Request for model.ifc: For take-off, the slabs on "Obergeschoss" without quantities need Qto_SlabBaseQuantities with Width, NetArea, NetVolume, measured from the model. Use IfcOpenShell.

First a look at what the model holds.

```python
import ifcopenshell
import ifcopenshell.util.element
import ifcopenshell.util.unit

model = ifcopenshell.open("model.ifc")
print(model.schema)
for unit_type in ("LENGTHUNIT", "AREAUNIT", "VOLUMEUNIT"):
    print(unit_type, ifcopenshell.util.unit.calculate_unit_scale(model, unit_type))
storey = next(s for s in model.by_type("IfcBuildingStorey") if s.Name == "Obergeschoss")
slabs = [e for e in ifcopenshell.util.element.get_decomposition(storey) if e.is_a("IfcSlab")]
for e in sorted(slabs, key=lambda e: e.id()):
    print(e.id(), e.is_a(), e.Name, list(ifcopenshell.util.element.get_psets(e, qtos_only=True)), sep=" | ")
```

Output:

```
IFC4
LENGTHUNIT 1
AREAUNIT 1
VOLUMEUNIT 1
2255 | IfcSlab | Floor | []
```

```python
import ifcopenshell
import ifcopenshell.api.pset
import ifcopenshell.geom
import ifcopenshell.util.element
import ifcopenshell.util.shape
import ifcopenshell.util.unit

model = ifcopenshell.open("model.ifc")
unit_scale = ifcopenshell.util.unit.calculate_unit_scale(model)
area_scale = ifcopenshell.util.unit.calculate_unit_scale(model, "AREAUNIT")
volume_scale = ifcopenshell.util.unit.calculate_unit_scale(model, "VOLUMEUNIT")
settings = ifcopenshell.geom.settings()

storey = next(s for s in model.by_type("IfcBuildingStorey") if s.Name == "Obergeschoss")
slabs = [e for e in ifcopenshell.util.element.get_decomposition(storey) if e.is_a("IfcSlab")]

for e in sorted(slabs, key=lambda e: e.id()):
    if ifcopenshell.util.element.get_psets(e, qtos_only=True, should_inherit=False):
        continue
    # Geometry comes back in metres, in the element's own axes.
    shape = ifcopenshell.geom.create_shape(settings, e)
    values = {
        "Width": ifcopenshell.util.shape.get_z(shape.geometry) / unit_scale,
        "NetArea": ifcopenshell.util.shape.get_footprint_area(shape.geometry) / area_scale,
        "NetVolume": ifcopenshell.util.shape.get_volume(shape.geometry) / volume_scale,
    }
    qto = ifcopenshell.api.pset.add_qto(model, product=e, name="Qto_SlabBaseQuantities")
    ifcopenshell.api.pset.edit_qto(model, qto=qto, properties=values)
    print(e.id(), {k: round(v, 3) for k, v in values.items()})

model.write("model_rev.ifc")
```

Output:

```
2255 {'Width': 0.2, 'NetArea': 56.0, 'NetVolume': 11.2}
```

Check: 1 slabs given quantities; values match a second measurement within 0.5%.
